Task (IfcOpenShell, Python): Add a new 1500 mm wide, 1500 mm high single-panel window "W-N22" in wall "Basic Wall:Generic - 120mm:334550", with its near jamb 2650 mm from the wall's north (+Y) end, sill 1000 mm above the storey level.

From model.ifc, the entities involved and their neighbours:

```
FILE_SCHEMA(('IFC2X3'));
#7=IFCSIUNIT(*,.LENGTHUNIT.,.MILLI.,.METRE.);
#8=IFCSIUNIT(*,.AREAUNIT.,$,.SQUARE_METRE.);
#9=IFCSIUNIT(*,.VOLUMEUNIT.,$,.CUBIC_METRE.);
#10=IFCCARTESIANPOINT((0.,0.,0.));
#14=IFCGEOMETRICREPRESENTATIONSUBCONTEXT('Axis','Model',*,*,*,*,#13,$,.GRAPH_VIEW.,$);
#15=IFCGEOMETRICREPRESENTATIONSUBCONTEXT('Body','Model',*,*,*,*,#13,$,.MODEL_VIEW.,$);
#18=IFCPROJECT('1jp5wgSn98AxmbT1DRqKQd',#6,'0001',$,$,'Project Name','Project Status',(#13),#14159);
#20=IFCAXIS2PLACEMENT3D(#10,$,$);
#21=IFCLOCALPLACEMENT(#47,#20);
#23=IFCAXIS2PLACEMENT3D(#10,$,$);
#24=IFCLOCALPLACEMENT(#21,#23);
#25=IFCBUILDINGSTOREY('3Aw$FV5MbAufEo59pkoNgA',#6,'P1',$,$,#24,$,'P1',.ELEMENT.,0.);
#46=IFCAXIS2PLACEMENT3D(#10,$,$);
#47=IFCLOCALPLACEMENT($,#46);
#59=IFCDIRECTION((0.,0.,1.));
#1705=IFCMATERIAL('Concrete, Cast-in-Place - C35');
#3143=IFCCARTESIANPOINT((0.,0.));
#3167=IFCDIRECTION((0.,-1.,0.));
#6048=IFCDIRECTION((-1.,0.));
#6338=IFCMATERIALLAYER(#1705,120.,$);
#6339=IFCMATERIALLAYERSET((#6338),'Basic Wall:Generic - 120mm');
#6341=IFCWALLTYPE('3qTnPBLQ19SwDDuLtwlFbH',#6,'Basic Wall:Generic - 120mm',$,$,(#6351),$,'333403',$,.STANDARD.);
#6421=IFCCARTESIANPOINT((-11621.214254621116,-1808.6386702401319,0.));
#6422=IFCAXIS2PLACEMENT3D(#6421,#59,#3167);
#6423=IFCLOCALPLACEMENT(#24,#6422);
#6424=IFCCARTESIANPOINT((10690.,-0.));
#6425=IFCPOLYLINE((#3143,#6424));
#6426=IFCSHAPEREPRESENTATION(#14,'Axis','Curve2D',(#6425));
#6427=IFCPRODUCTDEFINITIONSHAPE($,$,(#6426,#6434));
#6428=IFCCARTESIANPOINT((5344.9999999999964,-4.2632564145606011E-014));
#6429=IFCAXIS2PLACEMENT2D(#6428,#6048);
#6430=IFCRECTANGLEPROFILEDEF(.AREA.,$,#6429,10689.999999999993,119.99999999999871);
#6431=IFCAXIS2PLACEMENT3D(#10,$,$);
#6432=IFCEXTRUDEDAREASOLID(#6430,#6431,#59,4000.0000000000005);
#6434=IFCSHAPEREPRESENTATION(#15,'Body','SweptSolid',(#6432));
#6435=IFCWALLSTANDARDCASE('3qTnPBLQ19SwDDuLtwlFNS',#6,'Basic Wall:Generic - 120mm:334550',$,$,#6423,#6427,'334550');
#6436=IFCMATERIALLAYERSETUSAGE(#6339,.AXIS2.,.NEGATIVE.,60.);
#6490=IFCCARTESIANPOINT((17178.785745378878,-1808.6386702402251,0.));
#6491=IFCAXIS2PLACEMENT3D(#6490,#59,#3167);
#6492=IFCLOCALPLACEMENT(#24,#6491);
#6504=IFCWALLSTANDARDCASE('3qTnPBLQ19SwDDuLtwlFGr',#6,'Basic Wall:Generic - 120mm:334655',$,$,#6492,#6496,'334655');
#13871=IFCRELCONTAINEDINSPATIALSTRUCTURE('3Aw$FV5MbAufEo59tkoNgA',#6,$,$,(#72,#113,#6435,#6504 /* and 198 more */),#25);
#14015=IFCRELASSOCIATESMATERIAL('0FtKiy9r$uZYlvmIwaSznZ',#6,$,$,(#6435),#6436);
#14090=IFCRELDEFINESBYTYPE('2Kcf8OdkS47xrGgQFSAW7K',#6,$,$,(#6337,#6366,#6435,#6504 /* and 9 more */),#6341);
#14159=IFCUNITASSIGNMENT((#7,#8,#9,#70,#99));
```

```python
import numpy as np
import ifcopenshell
import ifcopenshell.api.feature
import ifcopenshell.api.geometry
import ifcopenshell.api.root
import ifcopenshell.api.spatial
import ifcopenshell.api.type
import ifcopenshell.geom
import ifcopenshell.util.element
import ifcopenshell.util.placement
import ifcopenshell.util.representation
import ifcopenshell.util.shape
import ifcopenshell.util.unit

model = ifcopenshell.open("model.ifc")
unit_scale = ifcopenshell.util.unit.calculate_unit_scale(model)
settings = ifcopenshell.geom.settings()


def volume(element):
    """Net volume in cubic metres, openings subtracted."""
    shape = ifcopenshell.geom.create_shape(settings, element)
    return ifcopenshell.util.shape.get_volume(shape.geometry)


wall = model.by_guid("3qTnPBLQ19SwDDuLtwlFNS")
storey = ifcopenshell.util.element.get_container(wall, ifc_class="IfcBuildingStorey")
context = ifcopenshell.util.representation.get_context(model, "Model", "Body", "MODEL_VIEW")
before = volume(wall)

width, height, from_end, sill = 1.5, 1.5, 2.65, 1  # metres

# The wall runs along its own X axis, and the end named is its -X end.
wall_shape = ifcopenshell.geom.create_shape(settings, wall)
x, y, z = ifcopenshell.util.shape.get_vertices(wall_shape.geometry).T
start = x.min() + from_end
face, thickness = float(y.min()), float(y.max() - y.min())
wall_matrix = ifcopenshell.util.placement.get_local_placement(wall.ObjectPlacement)
level = ifcopenshell.util.placement.get_local_placement(storey.ObjectPlacement)[2, 3]


def in_wall(x, y):
    """Placement at x, y metres in the wall's axes, at sill height."""
    matrix = wall_matrix.copy()
    matrix[:, 3] = wall_matrix @ np.array([x / unit_scale, y / unit_scale, 0.0, 1.0])
    matrix[2, 3] = level + sill / unit_scale
    return matrix


# Opening: a box that overshoots both wall faces by 50 mm.
opening = ifcopenshell.api.root.create_entity(model, ifc_class="IfcOpeningElement")
box = ifcopenshell.api.geometry.add_wall_representation(
    model, context=context, length=width, height=height, thickness=thickness + 0.1
)
ifcopenshell.api.geometry.assign_representation(model, product=opening, representation=box)
ifcopenshell.api.geometry.edit_object_placement(model, product=opening, matrix=in_wall(start, face - 0.05), is_si=False)
ifcopenshell.api.feature.add_feature(model, feature=opening, element=wall)

window = ifcopenshell.api.root.create_entity(model, ifc_class="IfcWindow", name="W-N22")
window.OverallWidth, window.OverallHeight = width / unit_scale, height / unit_scale
body = ifcopenshell.api.geometry.add_window_representation(
    model,
    context=context,
    overall_width=window.OverallWidth,
    overall_height=window.OverallHeight,
    partition_type="SINGLE_PANEL",
)
ifcopenshell.api.geometry.assign_representation(model, product=window, representation=body)
ifcopenshell.api.spatial.assign_container(model, products=[window], relating_structure=storey)
fills = ifcopenshell.api.feature.add_filling(model, opening=opening, element=window)
fills.OwnerHistory = window.OwnerHistory  # required in IFC2X3

# IFC2X3 keeps the operation on the window style.
style = ifcopenshell.api.root.create_entity(model, ifc_class="IfcWindowStyle", name="W-N22")
style.OperationType, style.ConstructionType = "SINGLE_PANEL", "NOTDEFINED"
style.ParameterTakesPrecedence = style.Sizeable = False
ifcopenshell.api.type.assign_type(model, related_objects=[window], relating_type=style)

# Centre the window in the wall's thickness.
ifcopenshell.api.geometry.edit_object_placement(model, product=window, matrix=in_wall(start, face), is_si=False)
window_shape = ifcopenshell.geom.create_shape(settings, window)
depth = ifcopenshell.util.shape.get_vertices(window_shape.geometry)[:, 1]
offset = face + thickness / 2 - (depth.min() + depth.max()) / 2
ifcopenshell.api.geometry.edit_object_placement(model, product=window, matrix=in_wall(start, offset), is_si=False)

after = volume(wall)

print(f"wall volume {before:.3f} -> {after:.3f} m3")

model.write("model-out.ifc")
```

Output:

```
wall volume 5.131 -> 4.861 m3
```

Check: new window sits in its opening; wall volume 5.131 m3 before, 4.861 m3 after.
